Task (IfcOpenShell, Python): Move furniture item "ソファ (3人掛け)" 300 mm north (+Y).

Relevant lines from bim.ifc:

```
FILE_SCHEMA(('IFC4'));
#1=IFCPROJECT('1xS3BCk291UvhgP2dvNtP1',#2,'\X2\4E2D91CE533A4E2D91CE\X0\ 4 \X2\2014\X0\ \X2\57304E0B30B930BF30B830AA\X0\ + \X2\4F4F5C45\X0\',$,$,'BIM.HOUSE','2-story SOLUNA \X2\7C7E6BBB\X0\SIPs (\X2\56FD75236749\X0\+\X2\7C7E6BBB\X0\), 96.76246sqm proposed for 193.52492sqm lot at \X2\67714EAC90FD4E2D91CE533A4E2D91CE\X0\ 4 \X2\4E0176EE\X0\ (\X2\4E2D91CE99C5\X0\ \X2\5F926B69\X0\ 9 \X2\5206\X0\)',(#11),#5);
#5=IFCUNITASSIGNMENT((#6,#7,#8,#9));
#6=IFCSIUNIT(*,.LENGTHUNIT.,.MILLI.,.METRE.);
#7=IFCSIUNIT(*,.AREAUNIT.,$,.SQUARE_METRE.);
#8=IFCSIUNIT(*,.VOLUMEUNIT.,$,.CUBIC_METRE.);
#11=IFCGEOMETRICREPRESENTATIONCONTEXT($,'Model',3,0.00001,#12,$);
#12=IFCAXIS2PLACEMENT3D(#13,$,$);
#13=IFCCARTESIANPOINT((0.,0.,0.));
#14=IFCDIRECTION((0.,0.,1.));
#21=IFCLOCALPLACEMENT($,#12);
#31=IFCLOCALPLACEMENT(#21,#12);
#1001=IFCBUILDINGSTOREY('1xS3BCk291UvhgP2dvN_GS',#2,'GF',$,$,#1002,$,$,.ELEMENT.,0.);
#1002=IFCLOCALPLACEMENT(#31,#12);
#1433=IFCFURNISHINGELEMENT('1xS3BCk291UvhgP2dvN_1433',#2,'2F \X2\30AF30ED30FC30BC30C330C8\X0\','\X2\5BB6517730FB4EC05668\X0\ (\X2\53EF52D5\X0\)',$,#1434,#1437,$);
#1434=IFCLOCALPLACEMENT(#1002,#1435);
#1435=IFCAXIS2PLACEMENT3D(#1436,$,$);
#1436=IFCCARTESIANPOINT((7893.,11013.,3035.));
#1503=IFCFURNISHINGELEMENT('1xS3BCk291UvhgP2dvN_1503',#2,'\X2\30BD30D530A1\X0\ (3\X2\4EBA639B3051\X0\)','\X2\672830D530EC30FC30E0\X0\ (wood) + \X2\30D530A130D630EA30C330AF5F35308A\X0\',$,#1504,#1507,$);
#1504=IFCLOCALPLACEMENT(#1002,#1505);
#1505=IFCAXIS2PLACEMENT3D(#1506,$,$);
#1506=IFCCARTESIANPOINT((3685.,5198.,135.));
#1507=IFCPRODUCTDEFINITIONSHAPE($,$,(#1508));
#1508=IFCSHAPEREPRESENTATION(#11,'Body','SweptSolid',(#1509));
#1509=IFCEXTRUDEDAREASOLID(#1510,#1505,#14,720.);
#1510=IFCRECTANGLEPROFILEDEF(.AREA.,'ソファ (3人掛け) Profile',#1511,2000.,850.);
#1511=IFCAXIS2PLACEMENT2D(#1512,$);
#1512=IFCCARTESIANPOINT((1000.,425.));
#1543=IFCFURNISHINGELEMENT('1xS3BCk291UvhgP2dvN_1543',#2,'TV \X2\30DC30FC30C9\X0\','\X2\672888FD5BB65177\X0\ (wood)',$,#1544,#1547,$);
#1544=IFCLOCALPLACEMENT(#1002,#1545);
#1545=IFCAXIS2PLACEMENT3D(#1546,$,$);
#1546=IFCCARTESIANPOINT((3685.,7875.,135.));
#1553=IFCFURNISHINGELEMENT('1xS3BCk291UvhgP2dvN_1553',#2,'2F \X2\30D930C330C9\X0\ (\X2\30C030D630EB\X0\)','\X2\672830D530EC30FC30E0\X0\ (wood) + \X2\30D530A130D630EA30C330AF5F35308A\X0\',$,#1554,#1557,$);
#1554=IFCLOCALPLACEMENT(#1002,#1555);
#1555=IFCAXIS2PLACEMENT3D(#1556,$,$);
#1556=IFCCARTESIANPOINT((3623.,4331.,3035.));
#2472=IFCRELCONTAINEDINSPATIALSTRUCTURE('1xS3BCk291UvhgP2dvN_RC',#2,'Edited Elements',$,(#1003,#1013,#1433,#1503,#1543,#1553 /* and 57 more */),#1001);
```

```python
import ifcopenshell
import ifcopenshell.api.geometry
import ifcopenshell.util.placement
import ifcopenshell.util.unit

model = ifcopenshell.open("bim.ifc")
unit_scale = ifcopenshell.util.unit.calculate_unit_scale(model)

item = model.by_guid("1xS3BCk291UvhgP2dvN_1503")
matrix = ifcopenshell.util.placement.get_local_placement(item.ObjectPlacement)
matrix[1, 3] += 0.3 / unit_scale
ifcopenshell.api.geometry.edit_object_placement(model, product=item, matrix=matrix, is_si=False)

print(ifcopenshell.util.placement.get_local_placement(item.ObjectPlacement).round(3) + 0.0)

model.write("bim_rev.ifc")
```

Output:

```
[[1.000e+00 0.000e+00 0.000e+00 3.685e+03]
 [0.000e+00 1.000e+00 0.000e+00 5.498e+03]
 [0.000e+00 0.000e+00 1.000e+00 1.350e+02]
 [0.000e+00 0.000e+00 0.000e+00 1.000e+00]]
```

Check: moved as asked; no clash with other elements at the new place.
